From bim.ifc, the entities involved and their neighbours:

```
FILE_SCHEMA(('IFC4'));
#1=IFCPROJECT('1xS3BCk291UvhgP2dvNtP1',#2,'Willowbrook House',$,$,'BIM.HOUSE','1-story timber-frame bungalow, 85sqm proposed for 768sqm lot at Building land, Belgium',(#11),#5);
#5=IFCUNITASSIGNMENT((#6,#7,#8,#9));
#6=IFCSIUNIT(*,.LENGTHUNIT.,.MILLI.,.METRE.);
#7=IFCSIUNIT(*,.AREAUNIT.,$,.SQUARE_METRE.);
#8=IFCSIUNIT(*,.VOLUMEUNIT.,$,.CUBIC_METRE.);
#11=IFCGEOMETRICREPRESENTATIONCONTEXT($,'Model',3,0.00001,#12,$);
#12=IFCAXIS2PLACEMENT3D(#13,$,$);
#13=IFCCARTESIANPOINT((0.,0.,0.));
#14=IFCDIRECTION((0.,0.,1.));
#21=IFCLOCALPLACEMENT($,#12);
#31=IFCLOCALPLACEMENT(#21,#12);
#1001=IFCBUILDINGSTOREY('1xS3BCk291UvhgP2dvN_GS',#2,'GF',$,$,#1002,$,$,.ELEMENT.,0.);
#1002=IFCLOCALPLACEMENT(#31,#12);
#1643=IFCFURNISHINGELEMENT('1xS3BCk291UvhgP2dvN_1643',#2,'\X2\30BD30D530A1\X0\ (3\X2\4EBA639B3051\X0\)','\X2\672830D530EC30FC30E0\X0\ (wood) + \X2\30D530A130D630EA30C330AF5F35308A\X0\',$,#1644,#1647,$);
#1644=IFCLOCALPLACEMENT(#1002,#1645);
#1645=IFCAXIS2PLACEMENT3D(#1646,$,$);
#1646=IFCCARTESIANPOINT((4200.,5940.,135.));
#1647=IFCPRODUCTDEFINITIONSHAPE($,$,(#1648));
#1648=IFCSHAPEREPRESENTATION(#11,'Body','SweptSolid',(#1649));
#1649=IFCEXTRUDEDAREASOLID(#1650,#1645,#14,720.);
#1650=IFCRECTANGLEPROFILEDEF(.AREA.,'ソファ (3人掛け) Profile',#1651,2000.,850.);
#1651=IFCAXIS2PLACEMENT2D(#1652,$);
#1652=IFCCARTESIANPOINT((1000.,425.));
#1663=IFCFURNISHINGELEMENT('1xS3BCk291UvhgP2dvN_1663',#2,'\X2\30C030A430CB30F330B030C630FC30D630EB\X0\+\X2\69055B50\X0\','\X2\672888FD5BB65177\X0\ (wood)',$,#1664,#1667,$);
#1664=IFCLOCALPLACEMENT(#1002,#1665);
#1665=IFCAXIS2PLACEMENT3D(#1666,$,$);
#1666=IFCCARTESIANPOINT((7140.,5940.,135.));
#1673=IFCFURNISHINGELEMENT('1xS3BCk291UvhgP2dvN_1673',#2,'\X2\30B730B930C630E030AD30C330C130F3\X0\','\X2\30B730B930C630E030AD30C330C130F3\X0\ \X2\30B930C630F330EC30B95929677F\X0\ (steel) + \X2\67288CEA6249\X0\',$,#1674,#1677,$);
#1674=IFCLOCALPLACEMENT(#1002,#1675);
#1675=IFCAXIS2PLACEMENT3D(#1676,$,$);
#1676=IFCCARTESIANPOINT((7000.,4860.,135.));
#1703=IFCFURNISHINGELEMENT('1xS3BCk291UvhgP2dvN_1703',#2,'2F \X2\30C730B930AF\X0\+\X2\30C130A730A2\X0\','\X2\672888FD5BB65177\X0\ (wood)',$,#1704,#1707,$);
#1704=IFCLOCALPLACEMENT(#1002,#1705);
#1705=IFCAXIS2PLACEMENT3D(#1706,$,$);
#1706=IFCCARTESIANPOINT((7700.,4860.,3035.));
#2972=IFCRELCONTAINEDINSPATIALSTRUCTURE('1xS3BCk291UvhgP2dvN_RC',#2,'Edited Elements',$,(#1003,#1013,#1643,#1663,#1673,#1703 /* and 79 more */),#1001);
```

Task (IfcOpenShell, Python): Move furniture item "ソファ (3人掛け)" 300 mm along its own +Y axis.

```python
import ifcopenshell
import ifcopenshell.api.geometry
import ifcopenshell.util.placement

model = ifcopenshell.open("bim.ifc")

item = model.by_guid("1xS3BCk291UvhgP2dvN_1643")
matrix = ifcopenshell.util.placement.get_local_placement(item.ObjectPlacement)
matrix[:3, 3] += matrix[:3, 1] * 300.0
ifcopenshell.api.geometry.edit_object_placement(model, product=item, matrix=matrix, is_si=False)

print(ifcopenshell.util.placement.get_local_placement(item.ObjectPlacement).round(3) + 0.0)

model.write("bim_v2.ifc")
```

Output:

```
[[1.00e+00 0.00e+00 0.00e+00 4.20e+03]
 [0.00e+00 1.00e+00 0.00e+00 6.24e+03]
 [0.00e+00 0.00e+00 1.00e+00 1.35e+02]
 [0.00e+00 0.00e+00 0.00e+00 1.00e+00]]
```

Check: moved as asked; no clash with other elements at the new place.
